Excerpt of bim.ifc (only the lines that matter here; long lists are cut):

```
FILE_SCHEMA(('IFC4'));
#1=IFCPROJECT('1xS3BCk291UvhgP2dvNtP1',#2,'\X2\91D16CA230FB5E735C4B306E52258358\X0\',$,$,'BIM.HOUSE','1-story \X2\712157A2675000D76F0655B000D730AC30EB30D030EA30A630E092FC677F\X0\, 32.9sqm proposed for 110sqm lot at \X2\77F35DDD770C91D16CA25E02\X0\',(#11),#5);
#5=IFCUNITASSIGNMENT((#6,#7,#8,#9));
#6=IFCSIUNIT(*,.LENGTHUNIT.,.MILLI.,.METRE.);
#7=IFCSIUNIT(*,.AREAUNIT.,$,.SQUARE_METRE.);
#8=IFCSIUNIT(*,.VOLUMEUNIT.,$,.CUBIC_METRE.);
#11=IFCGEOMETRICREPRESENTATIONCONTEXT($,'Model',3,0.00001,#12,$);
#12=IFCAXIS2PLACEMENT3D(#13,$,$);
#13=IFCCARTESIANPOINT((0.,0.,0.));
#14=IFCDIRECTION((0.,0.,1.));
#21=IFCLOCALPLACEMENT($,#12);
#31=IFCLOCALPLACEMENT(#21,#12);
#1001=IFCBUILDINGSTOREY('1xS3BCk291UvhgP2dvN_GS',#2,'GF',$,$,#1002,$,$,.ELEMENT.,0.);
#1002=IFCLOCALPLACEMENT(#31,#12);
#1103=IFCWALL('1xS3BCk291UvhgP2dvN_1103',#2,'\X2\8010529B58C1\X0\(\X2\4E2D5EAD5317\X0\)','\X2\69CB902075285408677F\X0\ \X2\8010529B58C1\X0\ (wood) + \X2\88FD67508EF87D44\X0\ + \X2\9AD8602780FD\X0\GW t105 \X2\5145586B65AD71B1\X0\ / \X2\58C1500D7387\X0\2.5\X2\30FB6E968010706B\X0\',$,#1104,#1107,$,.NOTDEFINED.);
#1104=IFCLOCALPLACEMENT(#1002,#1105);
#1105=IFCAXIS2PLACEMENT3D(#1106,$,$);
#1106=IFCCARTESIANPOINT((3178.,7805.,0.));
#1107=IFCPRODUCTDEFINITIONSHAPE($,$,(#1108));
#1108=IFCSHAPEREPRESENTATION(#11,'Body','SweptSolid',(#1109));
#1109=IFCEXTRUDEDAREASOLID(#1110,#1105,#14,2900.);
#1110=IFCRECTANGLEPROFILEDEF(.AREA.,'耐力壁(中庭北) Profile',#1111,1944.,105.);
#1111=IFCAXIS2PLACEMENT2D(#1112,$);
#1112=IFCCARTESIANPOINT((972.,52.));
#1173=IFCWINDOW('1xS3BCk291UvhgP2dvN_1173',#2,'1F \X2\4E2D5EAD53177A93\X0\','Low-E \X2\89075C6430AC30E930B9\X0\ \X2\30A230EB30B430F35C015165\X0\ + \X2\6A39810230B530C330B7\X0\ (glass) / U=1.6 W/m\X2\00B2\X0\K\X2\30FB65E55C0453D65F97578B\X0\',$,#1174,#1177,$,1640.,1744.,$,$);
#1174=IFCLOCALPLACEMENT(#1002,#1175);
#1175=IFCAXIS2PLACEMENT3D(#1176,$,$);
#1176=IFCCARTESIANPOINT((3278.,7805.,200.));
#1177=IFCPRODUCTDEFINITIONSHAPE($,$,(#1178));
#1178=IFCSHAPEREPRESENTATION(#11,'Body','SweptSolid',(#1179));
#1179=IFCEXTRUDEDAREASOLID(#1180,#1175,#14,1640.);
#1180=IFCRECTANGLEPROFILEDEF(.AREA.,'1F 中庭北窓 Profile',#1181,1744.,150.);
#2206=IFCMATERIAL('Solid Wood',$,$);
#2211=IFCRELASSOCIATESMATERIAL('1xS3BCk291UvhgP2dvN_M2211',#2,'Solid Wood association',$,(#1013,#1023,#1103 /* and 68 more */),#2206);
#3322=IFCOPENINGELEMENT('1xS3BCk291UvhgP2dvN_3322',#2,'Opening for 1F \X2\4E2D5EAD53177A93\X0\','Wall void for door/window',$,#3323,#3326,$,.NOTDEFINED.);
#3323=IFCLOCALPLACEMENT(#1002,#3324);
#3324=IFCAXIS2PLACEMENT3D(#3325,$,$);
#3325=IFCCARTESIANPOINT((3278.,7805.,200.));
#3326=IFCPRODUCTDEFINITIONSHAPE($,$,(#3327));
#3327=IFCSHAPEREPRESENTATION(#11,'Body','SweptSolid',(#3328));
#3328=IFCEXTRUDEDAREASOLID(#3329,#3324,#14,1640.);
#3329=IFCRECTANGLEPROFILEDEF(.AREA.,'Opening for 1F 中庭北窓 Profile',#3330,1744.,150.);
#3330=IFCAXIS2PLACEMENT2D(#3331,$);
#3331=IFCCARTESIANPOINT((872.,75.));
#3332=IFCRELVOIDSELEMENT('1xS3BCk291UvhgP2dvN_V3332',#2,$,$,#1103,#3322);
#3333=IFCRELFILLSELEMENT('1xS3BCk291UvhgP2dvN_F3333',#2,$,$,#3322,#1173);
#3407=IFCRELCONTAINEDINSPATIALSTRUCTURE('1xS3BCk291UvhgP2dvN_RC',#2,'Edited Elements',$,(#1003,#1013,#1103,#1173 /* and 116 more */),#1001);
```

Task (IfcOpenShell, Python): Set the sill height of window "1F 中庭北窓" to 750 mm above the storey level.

```python
import numpy as np
import ifcopenshell
import ifcopenshell.api.geometry
import ifcopenshell.geom
import ifcopenshell.util.element
import ifcopenshell.util.placement
import ifcopenshell.util.shape
import ifcopenshell.util.unit

model = ifcopenshell.open("bim.ifc")
unit_scale = ifcopenshell.util.unit.calculate_unit_scale(model)

window = model.by_guid("1xS3BCk291UvhgP2dvN_1173")
opening = window.FillsVoids[0].RelatingOpeningElement
storey = ifcopenshell.util.element.get_container(window, ifc_class="IfcBuildingStorey")
level = ifcopenshell.util.placement.get_local_placement(storey.ObjectPlacement)[2, 3]

# The opening's origin need not be at the sill, so measure its lowest point.
shape = ifcopenshell.geom.create_shape(ifcopenshell.geom.settings(), opening)
bottom = ifcopenshell.util.shape.get_shape_bottom_elevation(shape, shape.geometry) / unit_scale
dz = level + 0.75 / unit_scale - bottom

shift = np.array([0.0, 0.0, dz])
# The window is not placed relative to its opening, so move both.
for product in (opening, window):
    matrix = ifcopenshell.util.placement.get_local_placement(product.ObjectPlacement)
    matrix[:3, 3] += shift
    ifcopenshell.api.geometry.edit_object_placement(model, product=product, matrix=matrix, is_si=False)

print(f"moved by {dz * unit_scale:+.3f} m")

model.write("bim_v2.ifc")
```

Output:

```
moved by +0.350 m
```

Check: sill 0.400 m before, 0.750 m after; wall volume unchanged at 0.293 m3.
